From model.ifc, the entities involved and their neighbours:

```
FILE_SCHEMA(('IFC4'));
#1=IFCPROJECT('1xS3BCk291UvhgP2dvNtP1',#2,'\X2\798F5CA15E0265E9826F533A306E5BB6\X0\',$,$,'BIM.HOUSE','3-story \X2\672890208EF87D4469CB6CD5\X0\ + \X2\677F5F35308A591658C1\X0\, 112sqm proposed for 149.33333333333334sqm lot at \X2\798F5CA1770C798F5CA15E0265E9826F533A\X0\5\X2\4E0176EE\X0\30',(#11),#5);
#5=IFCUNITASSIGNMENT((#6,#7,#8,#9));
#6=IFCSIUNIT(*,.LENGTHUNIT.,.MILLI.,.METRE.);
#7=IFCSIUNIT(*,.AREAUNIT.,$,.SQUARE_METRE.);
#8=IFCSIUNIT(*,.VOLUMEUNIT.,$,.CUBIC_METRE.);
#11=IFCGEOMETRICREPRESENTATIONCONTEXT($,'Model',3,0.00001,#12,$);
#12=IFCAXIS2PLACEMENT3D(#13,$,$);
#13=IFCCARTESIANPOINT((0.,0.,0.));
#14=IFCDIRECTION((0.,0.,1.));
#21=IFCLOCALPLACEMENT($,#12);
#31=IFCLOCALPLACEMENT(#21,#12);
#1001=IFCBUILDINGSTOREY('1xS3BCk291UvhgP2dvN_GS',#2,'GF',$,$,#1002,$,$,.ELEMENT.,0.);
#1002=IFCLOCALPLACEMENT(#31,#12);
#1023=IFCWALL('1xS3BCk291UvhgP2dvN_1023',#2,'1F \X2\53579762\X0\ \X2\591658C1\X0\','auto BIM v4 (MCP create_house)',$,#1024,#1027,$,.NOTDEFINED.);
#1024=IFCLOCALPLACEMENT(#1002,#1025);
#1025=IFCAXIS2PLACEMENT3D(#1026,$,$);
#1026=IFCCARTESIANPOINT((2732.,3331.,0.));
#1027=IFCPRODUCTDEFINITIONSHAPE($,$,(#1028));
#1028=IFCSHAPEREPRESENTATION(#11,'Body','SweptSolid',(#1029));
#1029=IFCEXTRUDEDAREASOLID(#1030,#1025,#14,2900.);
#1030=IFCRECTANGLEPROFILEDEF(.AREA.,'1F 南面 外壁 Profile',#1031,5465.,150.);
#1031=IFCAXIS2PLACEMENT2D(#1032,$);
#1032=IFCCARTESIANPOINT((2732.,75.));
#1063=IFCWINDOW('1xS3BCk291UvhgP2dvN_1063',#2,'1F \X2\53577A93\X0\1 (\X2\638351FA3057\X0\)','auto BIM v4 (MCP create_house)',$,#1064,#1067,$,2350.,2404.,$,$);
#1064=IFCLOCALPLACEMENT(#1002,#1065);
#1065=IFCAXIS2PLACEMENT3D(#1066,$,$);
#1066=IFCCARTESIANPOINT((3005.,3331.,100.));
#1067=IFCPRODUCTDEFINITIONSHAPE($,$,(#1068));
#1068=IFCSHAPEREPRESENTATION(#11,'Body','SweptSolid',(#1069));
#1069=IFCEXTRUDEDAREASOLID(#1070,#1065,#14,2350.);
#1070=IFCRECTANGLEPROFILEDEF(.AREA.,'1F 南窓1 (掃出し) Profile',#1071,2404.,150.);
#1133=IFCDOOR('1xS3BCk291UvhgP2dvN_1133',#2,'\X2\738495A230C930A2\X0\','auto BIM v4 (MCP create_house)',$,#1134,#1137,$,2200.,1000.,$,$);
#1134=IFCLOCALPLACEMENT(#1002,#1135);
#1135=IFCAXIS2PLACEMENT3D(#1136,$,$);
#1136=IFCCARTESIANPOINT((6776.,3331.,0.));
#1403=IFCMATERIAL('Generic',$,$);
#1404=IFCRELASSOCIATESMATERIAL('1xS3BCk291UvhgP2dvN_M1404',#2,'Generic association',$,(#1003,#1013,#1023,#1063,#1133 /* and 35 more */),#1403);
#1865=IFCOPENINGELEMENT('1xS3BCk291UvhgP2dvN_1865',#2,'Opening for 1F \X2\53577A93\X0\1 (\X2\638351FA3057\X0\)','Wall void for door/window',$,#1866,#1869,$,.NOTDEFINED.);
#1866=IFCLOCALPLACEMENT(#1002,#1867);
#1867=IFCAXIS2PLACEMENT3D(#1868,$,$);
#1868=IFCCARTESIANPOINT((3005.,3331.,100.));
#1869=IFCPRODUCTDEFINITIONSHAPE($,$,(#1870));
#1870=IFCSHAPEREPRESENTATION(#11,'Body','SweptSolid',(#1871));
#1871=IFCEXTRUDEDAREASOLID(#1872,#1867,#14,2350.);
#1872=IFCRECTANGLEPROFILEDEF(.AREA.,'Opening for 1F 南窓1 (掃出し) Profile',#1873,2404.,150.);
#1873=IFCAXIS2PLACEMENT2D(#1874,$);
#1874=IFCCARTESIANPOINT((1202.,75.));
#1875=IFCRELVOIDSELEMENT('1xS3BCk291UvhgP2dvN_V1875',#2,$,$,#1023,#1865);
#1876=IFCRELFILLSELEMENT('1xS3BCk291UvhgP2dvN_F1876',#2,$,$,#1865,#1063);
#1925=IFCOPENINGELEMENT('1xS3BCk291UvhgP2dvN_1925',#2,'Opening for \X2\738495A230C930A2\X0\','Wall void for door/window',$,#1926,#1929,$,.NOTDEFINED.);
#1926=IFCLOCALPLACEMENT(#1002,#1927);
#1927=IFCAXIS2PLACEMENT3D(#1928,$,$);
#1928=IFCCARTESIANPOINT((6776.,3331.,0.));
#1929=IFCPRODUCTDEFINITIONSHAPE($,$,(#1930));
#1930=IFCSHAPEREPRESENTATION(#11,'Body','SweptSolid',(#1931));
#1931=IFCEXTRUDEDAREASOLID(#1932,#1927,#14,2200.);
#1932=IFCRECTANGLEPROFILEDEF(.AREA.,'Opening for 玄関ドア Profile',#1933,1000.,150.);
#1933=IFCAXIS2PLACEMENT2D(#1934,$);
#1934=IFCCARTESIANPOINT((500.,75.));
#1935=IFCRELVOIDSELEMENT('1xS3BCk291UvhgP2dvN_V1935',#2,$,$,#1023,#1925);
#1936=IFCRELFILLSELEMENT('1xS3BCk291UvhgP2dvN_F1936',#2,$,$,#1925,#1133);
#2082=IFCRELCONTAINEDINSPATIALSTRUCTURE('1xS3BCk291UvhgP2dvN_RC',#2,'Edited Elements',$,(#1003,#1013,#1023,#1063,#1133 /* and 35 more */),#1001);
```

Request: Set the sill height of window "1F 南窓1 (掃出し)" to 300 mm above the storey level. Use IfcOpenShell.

```python
import numpy as np
import ifcopenshell
import ifcopenshell.api.geometry
import ifcopenshell.geom
import ifcopenshell.util.element
import ifcopenshell.util.placement
import ifcopenshell.util.shape
import ifcopenshell.util.unit

model = ifcopenshell.open("model.ifc")
unit_scale = ifcopenshell.util.unit.calculate_unit_scale(model)

window = model.by_guid("1xS3BCk291UvhgP2dvN_1063")
opening = window.FillsVoids[0].RelatingOpeningElement
storey = ifcopenshell.util.element.get_container(window, ifc_class="IfcBuildingStorey")
level = ifcopenshell.util.placement.get_local_placement(storey.ObjectPlacement)[2, 3]

# The opening's origin need not be at the sill, so measure its lowest point.
shape = ifcopenshell.geom.create_shape(ifcopenshell.geom.settings(), opening)
bottom = ifcopenshell.util.shape.get_shape_bottom_elevation(shape, shape.geometry) / unit_scale
dz = level + 0.3 / unit_scale - bottom

shift = np.array([0.0, 0.0, dz])
# The window is not placed relative to its opening, so move both.
for product in (opening, window):
    matrix = ifcopenshell.util.placement.get_local_placement(product.ObjectPlacement)
    matrix[:3, 3] += shift
    ifcopenshell.api.geometry.edit_object_placement(model, product=product, matrix=matrix, is_si=False)

print(f"moved by {dz * unit_scale:+.3f} m")

model.write("model_edited.ifc")
```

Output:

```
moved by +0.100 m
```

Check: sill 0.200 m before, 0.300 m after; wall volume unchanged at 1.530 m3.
